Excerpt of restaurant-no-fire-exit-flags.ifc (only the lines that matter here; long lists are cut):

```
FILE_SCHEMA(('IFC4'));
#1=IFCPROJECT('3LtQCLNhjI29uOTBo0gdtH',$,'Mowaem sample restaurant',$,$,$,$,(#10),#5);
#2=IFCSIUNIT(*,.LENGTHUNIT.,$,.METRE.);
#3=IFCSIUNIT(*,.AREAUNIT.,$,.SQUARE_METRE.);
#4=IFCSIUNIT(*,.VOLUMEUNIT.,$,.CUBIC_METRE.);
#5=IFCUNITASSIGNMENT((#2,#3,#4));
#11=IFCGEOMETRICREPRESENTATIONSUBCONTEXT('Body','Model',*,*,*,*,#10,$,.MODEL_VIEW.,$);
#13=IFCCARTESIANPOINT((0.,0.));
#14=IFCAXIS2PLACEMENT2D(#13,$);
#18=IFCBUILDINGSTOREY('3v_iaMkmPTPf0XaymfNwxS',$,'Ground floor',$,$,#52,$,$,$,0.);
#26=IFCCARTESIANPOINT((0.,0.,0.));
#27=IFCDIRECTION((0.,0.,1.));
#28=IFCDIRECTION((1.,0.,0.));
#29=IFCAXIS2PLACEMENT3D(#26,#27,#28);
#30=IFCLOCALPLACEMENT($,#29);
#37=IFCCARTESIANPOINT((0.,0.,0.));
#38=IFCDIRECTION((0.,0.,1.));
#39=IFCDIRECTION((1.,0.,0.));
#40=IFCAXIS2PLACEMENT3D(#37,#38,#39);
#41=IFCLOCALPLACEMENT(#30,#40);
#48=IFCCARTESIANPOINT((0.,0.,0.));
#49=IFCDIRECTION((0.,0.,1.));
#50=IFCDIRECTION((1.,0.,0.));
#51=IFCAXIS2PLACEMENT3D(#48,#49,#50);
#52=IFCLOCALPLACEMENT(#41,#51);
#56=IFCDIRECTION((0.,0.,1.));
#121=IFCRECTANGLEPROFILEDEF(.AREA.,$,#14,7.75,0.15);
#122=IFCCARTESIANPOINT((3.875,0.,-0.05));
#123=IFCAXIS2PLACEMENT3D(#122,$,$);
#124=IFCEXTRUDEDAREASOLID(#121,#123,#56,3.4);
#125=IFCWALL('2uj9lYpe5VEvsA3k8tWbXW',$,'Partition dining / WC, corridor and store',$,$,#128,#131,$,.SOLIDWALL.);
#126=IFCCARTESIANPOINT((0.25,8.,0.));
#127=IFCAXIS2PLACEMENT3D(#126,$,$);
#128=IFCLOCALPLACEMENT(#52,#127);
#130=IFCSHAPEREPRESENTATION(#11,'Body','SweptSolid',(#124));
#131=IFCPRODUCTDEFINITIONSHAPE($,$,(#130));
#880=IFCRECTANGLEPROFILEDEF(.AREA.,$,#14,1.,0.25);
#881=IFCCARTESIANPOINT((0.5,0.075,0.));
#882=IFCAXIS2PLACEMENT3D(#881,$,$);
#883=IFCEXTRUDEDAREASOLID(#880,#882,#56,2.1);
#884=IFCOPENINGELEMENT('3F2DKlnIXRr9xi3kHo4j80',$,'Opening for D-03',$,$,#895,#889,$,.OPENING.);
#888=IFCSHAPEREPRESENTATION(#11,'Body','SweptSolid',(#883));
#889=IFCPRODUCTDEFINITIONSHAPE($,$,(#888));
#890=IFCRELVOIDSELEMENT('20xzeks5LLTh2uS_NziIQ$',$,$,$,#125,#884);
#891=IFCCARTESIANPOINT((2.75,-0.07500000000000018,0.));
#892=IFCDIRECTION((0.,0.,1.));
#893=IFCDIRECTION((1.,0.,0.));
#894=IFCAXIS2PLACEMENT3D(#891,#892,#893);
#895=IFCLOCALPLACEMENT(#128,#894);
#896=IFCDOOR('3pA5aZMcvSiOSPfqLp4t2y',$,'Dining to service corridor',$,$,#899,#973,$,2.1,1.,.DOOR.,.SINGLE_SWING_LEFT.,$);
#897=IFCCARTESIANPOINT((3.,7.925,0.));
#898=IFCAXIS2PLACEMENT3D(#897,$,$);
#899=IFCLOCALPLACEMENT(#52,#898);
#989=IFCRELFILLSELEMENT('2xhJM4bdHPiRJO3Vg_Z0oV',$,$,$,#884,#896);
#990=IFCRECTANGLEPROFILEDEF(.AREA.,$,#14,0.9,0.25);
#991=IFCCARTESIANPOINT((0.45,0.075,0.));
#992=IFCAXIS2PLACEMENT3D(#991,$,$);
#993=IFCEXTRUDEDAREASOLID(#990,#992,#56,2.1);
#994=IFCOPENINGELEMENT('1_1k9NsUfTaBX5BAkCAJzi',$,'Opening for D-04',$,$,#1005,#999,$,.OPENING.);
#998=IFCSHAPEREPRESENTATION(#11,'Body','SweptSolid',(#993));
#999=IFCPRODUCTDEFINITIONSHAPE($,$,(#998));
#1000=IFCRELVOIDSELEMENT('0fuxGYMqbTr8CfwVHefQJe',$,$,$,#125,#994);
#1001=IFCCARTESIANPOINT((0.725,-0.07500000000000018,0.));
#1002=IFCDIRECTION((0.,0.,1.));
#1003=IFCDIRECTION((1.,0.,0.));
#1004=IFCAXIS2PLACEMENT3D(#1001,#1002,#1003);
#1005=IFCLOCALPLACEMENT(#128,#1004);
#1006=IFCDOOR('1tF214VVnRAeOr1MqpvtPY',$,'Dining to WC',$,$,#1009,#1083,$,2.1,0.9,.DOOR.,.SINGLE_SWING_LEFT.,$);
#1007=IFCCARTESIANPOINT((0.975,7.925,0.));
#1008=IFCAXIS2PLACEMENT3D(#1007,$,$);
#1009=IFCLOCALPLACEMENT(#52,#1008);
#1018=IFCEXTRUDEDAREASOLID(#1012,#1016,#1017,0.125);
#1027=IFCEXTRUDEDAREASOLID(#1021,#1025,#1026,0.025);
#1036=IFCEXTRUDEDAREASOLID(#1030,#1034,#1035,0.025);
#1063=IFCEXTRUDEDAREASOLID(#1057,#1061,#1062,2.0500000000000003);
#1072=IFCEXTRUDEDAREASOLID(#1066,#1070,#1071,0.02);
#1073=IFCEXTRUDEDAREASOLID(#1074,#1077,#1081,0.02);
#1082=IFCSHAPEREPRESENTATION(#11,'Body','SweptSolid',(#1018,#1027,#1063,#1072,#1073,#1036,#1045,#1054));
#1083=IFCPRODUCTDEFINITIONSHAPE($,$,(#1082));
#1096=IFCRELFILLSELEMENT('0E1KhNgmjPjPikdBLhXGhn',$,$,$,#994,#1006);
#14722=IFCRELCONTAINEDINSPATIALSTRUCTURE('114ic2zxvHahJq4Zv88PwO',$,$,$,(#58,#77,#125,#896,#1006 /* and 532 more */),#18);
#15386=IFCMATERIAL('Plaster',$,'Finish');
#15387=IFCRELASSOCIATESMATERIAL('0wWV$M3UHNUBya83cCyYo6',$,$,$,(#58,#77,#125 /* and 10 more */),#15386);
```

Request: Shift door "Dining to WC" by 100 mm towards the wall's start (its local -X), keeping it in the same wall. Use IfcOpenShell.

```python
import ifcopenshell
import ifcopenshell.api.geometry
import ifcopenshell.util.placement
import ifcopenshell.util.unit

model = ifcopenshell.open("restaurant-no-fire-exit-flags.ifc")
unit_scale = ifcopenshell.util.unit.calculate_unit_scale(model)

door = model.by_guid("1tF214VVnRAeOr1MqpvtPY")
opening = door.FillsVoids[0].RelatingOpeningElement
wall = opening.VoidsElements[0].RelatingBuildingElement

wall_matrix = ifcopenshell.util.placement.get_local_placement(wall.ObjectPlacement)
shift = wall_matrix[:3, 0] * -0.1 / unit_scale
before = ifcopenshell.util.placement.get_local_placement(door.ObjectPlacement)[:3, 3].copy()

# The door is not placed relative to its opening, so move both.
for product in (opening, door):
    matrix = ifcopenshell.util.placement.get_local_placement(product.ObjectPlacement)
    matrix[:3, 3] += shift
    ifcopenshell.api.geometry.edit_object_placement(model, product=product, matrix=matrix, is_si=False)

after = ifcopenshell.util.placement.get_local_placement(door.ObjectPlacement)[:3, 3]
print("door moved by", (after - before).round(3) + 0.0)

model.write("restaurant-no-fire-exit-flags_edited.ifc")
```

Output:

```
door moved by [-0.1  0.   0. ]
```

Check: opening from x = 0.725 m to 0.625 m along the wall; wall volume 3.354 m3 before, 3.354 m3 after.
